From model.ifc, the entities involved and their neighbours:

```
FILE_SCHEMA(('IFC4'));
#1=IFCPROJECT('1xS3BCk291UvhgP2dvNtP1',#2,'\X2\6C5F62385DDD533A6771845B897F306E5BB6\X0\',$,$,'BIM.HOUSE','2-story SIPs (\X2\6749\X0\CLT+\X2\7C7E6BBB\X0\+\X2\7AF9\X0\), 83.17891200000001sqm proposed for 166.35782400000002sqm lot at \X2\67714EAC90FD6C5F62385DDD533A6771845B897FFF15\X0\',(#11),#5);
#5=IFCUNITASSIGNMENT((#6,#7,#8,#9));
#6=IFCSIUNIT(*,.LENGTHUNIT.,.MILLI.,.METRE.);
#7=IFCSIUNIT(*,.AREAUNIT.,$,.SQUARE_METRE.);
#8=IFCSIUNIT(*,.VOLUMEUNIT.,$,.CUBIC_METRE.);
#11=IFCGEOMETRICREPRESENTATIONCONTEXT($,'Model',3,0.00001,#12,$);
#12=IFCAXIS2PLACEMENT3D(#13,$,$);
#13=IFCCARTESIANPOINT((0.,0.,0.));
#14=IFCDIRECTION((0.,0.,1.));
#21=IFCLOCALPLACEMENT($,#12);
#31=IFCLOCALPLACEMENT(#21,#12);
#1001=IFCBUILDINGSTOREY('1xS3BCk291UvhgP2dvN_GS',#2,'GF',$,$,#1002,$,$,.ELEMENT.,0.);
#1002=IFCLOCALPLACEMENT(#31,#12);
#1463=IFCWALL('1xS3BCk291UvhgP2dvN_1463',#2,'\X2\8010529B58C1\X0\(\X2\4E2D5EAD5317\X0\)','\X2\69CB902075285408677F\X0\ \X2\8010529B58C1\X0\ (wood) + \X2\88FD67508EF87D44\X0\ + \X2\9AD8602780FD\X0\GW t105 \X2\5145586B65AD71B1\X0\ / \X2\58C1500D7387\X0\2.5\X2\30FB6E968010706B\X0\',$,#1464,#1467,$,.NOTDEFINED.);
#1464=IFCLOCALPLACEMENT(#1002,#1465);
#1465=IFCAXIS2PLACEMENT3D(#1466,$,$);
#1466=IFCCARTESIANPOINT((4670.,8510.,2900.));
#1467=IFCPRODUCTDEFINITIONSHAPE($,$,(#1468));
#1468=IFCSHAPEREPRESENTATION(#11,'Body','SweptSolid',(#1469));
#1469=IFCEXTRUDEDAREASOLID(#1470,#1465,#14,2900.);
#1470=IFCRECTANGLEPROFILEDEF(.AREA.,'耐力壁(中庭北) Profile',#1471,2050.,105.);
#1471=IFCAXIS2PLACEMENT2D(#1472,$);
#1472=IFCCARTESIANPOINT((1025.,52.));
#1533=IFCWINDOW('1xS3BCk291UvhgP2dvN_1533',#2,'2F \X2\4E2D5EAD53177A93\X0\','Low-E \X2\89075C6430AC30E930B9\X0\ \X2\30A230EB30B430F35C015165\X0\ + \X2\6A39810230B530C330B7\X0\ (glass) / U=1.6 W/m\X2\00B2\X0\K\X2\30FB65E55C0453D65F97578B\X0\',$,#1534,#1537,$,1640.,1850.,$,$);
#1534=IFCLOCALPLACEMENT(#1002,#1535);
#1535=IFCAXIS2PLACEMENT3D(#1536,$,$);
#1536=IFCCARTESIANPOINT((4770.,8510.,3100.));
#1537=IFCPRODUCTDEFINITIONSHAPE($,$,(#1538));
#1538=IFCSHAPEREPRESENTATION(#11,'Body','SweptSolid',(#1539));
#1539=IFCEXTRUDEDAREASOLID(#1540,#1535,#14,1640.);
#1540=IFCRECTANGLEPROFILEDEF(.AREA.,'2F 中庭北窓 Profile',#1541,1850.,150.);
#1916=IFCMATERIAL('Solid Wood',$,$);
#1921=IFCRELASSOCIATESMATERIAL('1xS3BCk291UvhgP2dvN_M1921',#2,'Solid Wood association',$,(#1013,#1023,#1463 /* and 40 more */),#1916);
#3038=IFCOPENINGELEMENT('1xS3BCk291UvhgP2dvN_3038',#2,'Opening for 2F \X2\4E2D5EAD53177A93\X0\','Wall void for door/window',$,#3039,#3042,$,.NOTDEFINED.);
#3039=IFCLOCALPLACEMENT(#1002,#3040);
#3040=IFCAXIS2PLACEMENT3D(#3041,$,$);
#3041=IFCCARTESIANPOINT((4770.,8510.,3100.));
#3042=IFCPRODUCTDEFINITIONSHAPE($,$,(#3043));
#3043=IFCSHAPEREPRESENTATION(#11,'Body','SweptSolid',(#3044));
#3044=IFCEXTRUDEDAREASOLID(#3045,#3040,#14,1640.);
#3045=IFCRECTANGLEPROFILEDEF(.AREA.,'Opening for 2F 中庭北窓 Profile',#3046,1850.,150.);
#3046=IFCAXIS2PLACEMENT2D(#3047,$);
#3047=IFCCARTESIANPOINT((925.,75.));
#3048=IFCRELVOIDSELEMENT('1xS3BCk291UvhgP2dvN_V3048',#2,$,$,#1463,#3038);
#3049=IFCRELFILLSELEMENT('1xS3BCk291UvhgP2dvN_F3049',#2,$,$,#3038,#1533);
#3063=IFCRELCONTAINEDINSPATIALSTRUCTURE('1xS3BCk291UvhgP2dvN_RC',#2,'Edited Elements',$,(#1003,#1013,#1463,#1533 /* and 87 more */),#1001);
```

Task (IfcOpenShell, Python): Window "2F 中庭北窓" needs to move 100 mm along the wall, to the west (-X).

```python
import ifcopenshell
import ifcopenshell.api.geometry
import ifcopenshell.util.placement
import ifcopenshell.util.unit

model = ifcopenshell.open("model.ifc")
unit_scale = ifcopenshell.util.unit.calculate_unit_scale(model)

window = model.by_id(1533)
opening = window.FillsVoids[0].RelatingOpeningElement
wall = opening.VoidsElements[0].RelatingBuildingElement

wall_matrix = ifcopenshell.util.placement.get_local_placement(wall.ObjectPlacement)
shift = wall_matrix[:3, 0] * -0.1 / unit_scale
before = ifcopenshell.util.placement.get_local_placement(window.ObjectPlacement)[:3, 3].copy()

# The window is not placed relative to its opening, so move both.
for product in (opening, window):
    matrix = ifcopenshell.util.placement.get_local_placement(product.ObjectPlacement)
    matrix[:3, 3] += shift
    ifcopenshell.api.geometry.edit_object_placement(model, product=product, matrix=matrix, is_si=False)

after = ifcopenshell.util.placement.get_local_placement(window.ObjectPlacement)[:3, 3]
print("window moved by", (after - before).round(3) + 0.0)

model.write("model_edited.ifc")
```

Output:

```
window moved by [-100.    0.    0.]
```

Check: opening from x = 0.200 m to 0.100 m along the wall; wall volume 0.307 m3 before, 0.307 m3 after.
